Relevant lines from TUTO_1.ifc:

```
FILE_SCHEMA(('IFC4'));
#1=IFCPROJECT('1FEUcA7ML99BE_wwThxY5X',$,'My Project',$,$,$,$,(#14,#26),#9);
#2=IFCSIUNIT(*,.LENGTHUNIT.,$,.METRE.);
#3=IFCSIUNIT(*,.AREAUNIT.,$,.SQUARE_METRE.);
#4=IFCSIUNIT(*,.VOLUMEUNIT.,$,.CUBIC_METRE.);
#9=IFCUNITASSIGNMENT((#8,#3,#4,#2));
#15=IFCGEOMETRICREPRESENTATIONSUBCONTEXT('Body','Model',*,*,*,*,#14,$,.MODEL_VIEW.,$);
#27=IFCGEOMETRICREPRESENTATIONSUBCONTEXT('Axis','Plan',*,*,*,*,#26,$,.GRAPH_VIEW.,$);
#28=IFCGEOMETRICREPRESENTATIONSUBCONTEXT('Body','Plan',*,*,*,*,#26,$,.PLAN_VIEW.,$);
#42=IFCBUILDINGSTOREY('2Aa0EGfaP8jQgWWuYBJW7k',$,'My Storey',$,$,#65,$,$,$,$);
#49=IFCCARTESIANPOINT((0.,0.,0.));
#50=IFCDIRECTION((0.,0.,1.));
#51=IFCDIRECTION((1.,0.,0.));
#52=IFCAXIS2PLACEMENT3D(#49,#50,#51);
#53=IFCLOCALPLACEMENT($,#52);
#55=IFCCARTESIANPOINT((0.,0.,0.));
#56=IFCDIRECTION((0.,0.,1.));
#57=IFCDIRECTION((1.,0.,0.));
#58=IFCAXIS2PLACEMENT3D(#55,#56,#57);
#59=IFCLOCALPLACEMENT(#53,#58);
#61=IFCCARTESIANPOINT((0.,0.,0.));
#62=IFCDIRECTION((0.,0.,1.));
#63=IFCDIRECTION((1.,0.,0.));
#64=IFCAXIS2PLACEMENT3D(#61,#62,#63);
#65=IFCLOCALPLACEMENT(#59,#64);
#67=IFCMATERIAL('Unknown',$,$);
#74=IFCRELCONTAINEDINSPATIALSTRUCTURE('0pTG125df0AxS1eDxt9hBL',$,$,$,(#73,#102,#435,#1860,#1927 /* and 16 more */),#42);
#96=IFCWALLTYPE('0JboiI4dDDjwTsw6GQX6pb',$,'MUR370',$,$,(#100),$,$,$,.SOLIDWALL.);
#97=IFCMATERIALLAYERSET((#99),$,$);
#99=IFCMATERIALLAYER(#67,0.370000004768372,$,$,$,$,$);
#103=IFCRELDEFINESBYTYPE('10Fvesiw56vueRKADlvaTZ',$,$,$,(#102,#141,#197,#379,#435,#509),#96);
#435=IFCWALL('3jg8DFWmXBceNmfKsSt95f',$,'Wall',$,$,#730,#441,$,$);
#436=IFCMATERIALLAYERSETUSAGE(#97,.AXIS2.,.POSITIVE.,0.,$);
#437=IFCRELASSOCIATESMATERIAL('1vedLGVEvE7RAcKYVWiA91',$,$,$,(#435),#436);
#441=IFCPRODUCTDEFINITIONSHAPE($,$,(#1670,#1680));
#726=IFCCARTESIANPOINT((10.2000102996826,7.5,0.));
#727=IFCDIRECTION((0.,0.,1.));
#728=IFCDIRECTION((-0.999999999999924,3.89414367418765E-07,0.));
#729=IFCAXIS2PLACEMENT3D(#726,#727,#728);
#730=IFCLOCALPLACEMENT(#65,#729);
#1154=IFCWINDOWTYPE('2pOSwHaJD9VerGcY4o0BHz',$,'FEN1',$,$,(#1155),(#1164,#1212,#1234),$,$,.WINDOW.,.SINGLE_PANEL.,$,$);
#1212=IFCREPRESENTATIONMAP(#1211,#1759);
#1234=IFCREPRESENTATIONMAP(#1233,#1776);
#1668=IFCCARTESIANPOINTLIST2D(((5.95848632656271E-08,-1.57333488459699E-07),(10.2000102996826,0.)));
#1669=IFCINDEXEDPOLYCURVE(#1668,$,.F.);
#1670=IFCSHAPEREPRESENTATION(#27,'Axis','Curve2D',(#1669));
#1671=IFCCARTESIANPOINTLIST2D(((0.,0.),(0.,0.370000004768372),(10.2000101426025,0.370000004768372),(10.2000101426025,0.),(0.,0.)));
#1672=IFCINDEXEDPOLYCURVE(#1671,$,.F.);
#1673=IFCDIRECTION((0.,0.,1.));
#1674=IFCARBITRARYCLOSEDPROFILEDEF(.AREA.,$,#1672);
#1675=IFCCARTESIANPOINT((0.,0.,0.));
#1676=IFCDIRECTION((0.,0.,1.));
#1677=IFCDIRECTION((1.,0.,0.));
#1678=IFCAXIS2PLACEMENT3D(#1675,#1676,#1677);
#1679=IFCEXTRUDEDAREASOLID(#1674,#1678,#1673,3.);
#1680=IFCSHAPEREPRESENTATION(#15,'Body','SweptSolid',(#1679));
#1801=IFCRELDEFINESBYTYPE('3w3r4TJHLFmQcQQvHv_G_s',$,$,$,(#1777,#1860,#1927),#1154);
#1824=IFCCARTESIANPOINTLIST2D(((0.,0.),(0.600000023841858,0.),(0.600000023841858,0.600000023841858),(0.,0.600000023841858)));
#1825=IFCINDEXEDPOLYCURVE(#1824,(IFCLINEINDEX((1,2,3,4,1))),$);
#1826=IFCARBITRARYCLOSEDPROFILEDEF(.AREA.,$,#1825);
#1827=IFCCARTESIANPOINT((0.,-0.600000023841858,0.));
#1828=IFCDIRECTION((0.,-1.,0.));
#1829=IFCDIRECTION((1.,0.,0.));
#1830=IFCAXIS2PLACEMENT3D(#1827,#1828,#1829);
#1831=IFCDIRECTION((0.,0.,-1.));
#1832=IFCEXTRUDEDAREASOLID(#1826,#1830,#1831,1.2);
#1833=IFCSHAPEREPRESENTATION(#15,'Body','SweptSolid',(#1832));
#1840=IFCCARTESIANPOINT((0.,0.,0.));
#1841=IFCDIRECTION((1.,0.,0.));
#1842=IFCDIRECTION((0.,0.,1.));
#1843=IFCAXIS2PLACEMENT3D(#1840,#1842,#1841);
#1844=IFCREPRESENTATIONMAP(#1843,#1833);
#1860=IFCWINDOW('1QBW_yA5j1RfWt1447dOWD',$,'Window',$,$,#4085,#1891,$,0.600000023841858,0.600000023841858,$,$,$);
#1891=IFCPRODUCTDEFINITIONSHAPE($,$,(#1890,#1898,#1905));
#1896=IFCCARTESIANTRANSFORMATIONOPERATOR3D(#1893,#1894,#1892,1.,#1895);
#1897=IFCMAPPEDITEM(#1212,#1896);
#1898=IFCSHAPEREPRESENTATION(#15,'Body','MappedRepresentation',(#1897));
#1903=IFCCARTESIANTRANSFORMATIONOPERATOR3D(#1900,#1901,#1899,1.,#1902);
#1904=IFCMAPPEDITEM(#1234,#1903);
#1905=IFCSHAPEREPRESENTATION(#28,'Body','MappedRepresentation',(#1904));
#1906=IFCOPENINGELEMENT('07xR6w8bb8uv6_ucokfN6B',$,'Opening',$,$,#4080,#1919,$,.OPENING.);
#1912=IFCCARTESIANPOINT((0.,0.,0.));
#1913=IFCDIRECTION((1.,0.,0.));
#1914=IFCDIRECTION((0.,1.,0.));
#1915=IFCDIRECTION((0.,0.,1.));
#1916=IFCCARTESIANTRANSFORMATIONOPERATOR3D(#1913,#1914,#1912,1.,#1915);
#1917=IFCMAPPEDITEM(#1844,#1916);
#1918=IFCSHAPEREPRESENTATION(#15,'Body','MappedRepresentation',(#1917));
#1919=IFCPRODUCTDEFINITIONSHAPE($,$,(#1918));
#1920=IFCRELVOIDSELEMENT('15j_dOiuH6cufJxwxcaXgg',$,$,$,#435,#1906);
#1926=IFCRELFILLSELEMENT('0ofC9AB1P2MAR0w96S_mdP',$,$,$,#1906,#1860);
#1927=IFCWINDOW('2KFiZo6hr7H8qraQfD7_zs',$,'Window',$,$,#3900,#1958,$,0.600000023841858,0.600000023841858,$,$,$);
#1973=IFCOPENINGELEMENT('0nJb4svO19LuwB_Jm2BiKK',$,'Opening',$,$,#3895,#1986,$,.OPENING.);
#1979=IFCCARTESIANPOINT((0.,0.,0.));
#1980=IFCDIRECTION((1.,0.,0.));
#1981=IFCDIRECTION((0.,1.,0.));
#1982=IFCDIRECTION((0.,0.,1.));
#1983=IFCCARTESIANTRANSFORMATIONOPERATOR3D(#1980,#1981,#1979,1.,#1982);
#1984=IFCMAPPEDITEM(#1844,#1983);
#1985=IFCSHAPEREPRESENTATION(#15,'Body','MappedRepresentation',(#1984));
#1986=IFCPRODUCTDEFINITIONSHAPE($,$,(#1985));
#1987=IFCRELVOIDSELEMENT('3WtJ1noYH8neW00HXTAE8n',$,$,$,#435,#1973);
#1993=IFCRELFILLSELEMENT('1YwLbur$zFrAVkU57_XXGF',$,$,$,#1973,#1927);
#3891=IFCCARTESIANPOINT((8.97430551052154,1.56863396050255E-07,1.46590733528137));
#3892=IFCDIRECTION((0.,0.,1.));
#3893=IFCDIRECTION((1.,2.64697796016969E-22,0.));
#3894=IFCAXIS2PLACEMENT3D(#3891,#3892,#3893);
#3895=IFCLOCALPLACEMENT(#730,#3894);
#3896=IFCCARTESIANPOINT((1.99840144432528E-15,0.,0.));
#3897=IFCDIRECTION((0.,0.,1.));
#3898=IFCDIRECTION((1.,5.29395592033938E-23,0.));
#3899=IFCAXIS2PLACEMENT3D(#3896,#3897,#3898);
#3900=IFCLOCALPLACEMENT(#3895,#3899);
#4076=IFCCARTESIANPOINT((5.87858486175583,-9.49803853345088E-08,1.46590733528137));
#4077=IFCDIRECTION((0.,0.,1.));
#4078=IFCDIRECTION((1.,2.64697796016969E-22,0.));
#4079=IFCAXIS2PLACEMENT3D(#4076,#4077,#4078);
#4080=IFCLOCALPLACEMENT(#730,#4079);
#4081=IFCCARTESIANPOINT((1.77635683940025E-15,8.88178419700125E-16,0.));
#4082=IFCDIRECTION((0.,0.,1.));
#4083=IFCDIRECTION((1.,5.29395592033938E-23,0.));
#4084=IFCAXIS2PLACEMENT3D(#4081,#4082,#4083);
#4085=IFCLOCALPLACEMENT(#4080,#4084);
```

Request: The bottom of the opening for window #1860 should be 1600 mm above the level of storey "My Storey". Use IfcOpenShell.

```python
import numpy as np
import ifcopenshell
import ifcopenshell.api.geometry
import ifcopenshell.geom
import ifcopenshell.util.element
import ifcopenshell.util.placement
import ifcopenshell.util.shape
import ifcopenshell.util.unit

model = ifcopenshell.open("TUTO_1.ifc")
unit_scale = ifcopenshell.util.unit.calculate_unit_scale(model)

window = model.by_guid("1QBW_yA5j1RfWt1447dOWD")
opening = window.FillsVoids[0].RelatingOpeningElement
storey = ifcopenshell.util.element.get_container(window, ifc_class="IfcBuildingStorey")
level = ifcopenshell.util.placement.get_local_placement(storey.ObjectPlacement)[2, 3]

# The opening's origin need not be at the sill, so measure its lowest point.
shape = ifcopenshell.geom.create_shape(ifcopenshell.geom.settings(), opening)
bottom = ifcopenshell.util.shape.get_shape_bottom_elevation(shape, shape.geometry) / unit_scale
dz = level + 1.6 / unit_scale - bottom

shift = np.array([0.0, 0.0, dz])
# The window is placed relative to its opening, so it follows when the opening moves.
matrix = ifcopenshell.util.placement.get_local_placement(opening.ObjectPlacement)
matrix[:3, 3] += shift
ifcopenshell.api.geometry.edit_object_placement(
    model, product=opening, matrix=matrix, is_si=False, should_transform_children=True
)

print(f"moved by {dz * unit_scale:+.3f} m")

model.write("TUTO_1_updated.ifc")
```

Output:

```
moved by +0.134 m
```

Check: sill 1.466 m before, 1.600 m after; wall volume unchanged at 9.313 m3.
